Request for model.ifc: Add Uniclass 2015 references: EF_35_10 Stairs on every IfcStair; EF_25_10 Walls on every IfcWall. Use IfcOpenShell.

First a look at what the model holds.

```python
import ifcopenshell

model = ifcopenshell.open("model.ifc")
print(model.schema)
print("classifications:", [c.Name for c in model.by_type("IfcClassification")])
for ifc_class in ("IfcDoor", "IfcRoof", "IfcStair", "IfcWall", "IfcWindow"):
    print(ifc_class, len(model.by_type(ifc_class)))
```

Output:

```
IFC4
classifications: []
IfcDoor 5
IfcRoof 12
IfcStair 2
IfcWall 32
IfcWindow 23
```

```python
import ifcopenshell
import ifcopenshell.api.classification

model = ifcopenshell.open("model.ifc")

system = ifcopenshell.api.classification.add_classification(model, classification="Uniclass 2015")

codes = {
    "IfcStair": ("EF_35_10", "Stairs"),
    "IfcWall": ("EF_25_10", "Walls"),
}
for ifc_class, (code, name) in codes.items():
    products = model.by_type(ifc_class)
    ifcopenshell.api.classification.add_reference(
        model, products=products, classification=system, identification=code, name=name
    )
    print(code, len(products))

model.write("model_edited.ifc")
```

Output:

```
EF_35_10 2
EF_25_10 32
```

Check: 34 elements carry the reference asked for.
